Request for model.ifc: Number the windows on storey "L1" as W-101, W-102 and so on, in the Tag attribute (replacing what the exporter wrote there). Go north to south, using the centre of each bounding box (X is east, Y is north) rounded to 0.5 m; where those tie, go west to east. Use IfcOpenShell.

First a look at what the model holds.

```python
import ifcopenshell
import ifcopenshell.util.element
import ifcopenshell.util.placement

model = ifcopenshell.open("model.ifc")
print(model.schema)
storey = next(s for s in model.by_type("IfcBuildingStorey") if s.Name == "L1")
windows = [e for e in ifcopenshell.util.element.get_decomposition(storey) if e.is_a("IfcWindow")]
for e in sorted(windows, key=lambda e: e.id()):
    origin = ifcopenshell.util.placement.get_local_placement(e.ObjectPlacement)[:3, 3]
    print(e.id(), e.Tag, e.Name, origin.round(2) + 0.0, sep=" | ")
```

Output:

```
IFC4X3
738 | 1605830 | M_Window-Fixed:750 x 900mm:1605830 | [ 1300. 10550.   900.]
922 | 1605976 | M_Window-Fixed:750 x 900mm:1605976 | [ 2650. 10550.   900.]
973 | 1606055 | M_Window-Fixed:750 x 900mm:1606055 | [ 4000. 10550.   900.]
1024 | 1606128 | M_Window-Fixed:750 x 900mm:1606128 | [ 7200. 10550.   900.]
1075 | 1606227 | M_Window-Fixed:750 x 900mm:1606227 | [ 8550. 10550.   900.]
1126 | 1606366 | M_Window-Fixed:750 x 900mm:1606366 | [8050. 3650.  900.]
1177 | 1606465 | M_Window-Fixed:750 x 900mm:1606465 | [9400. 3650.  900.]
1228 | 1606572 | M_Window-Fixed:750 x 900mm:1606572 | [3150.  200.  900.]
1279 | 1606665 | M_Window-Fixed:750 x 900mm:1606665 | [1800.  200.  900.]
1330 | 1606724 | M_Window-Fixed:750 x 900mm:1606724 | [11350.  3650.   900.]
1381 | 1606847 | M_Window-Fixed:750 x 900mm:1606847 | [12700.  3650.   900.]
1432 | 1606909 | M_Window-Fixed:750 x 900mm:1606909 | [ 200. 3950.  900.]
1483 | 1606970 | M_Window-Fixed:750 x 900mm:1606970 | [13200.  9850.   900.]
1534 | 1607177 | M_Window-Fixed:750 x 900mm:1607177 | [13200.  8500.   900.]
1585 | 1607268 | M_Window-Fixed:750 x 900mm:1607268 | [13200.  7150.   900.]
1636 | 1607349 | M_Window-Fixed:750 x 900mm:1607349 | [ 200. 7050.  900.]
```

```python
import ifcopenshell
import ifcopenshell.geom
import ifcopenshell.util.element
import ifcopenshell.util.shape

model = ifcopenshell.open("model.ifc")
settings = ifcopenshell.geom.settings()
settings.set("use-world-coords", True)


def centre(element):
    shape = ifcopenshell.geom.create_shape(settings, element)
    return ifcopenshell.util.shape.get_bbox_centroid(shape.geometry)


storey = next(s for s in model.by_type("IfcBuildingStorey") if s.Name == "L1")
windows = [e for e in ifcopenshell.util.element.get_decomposition(storey) if e.is_a("IfcWindow")]

# Insertion points can sit at a corner or the storey origin, so sort by the geometry (in metres).
centres = {e: centre(e) for e in windows}
windows.sort(key=lambda e: (-round(centres[e][1] / 0.5), centres[e][0]))

for i, e in enumerate(windows, start=1):
    number = f"W-1{i:02d}"
    e.Tag = number
    print(e.id(), number)

model.write("model_updated.ifc")
```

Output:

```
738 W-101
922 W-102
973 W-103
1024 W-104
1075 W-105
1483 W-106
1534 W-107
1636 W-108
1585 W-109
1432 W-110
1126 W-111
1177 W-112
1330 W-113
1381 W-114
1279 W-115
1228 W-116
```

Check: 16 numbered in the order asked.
